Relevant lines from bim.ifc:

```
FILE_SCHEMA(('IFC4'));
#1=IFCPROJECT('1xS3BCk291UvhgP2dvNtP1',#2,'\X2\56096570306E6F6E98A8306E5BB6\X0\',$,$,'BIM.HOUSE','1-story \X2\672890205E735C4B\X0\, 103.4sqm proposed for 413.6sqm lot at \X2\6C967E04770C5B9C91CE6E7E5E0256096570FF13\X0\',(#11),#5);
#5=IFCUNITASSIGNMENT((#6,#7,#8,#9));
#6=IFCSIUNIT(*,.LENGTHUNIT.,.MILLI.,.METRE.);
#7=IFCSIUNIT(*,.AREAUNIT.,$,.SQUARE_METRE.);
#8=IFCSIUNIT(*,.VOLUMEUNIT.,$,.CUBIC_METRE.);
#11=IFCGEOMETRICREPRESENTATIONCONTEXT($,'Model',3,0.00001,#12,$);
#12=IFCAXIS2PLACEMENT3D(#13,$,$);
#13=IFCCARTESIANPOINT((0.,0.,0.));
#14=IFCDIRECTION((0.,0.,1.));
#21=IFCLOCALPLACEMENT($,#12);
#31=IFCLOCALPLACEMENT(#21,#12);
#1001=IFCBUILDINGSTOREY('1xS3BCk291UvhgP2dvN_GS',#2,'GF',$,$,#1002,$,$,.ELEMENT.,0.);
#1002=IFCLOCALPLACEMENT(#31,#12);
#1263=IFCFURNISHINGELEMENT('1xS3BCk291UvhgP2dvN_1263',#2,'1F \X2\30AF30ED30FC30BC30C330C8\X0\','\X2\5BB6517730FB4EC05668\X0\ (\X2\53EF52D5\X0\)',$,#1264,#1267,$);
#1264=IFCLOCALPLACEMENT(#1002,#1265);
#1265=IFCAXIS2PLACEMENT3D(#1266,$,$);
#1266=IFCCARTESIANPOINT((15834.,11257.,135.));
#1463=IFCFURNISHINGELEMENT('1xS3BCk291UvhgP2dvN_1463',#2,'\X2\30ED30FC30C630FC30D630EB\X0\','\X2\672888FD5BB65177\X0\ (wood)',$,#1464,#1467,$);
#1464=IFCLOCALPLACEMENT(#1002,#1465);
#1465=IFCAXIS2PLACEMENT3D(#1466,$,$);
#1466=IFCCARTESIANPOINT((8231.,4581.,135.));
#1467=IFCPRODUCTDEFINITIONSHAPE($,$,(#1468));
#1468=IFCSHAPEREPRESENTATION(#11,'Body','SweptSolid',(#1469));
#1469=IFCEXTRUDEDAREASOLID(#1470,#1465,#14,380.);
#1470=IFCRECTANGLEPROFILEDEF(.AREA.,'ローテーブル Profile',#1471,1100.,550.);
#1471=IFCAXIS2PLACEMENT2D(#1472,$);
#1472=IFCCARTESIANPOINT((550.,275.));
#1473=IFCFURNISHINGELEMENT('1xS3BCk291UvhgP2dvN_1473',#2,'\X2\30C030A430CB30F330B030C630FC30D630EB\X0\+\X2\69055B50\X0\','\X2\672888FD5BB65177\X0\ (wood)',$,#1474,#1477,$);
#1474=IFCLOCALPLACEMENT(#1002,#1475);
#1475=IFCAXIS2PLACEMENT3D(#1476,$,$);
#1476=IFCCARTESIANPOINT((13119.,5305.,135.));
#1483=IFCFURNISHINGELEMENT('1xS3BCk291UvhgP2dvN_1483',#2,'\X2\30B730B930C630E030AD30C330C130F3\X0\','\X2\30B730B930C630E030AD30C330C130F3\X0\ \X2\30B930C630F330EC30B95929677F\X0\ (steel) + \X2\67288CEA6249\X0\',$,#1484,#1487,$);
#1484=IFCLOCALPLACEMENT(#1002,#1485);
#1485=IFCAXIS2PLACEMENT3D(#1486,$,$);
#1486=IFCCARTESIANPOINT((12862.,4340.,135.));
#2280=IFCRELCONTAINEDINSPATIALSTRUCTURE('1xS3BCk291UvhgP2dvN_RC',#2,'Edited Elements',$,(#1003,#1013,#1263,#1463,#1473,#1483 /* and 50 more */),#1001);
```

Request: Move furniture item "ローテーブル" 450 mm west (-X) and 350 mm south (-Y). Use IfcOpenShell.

```python
import ifcopenshell
import ifcopenshell.api.geometry
import ifcopenshell.util.placement

model = ifcopenshell.open("bim.ifc")

item = model.by_guid("1xS3BCk291UvhgP2dvN_1463")
matrix = ifcopenshell.util.placement.get_local_placement(item.ObjectPlacement)
matrix[0, 3] -= 450.0
matrix[1, 3] -= 350.0
ifcopenshell.api.geometry.edit_object_placement(model, product=item, matrix=matrix, is_si=False)

print(ifcopenshell.util.placement.get_local_placement(item.ObjectPlacement).round(3) + 0.0)

model.write("bim_v2.ifc")
```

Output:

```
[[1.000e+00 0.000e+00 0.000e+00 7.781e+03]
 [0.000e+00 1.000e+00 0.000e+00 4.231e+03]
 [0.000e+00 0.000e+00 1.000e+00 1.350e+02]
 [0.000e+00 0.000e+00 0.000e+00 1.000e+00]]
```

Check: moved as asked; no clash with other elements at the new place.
